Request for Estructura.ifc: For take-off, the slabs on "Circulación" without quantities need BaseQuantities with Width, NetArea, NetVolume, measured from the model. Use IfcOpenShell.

First a look at what the model holds.

```python
import ifcopenshell
import ifcopenshell.util.element
import ifcopenshell.util.unit

model = ifcopenshell.open("Estructura.ifc")
print(model.schema)
for unit_type in ("LENGTHUNIT", "AREAUNIT", "VOLUMEUNIT"):
    print(unit_type, ifcopenshell.util.unit.calculate_unit_scale(model, unit_type))
storey = next(s for s in model.by_type("IfcBuildingStorey") if s.Name == "Circulación")
slabs = [e for e in ifcopenshell.util.element.get_decomposition(storey) if e.is_a("IfcSlab")]
for e in sorted(slabs, key=lambda e: e.id()):
    print(e.id(), e.is_a(), e.Name, list(ifcopenshell.util.element.get_psets(e, qtos_only=True)), sep=" | ")
```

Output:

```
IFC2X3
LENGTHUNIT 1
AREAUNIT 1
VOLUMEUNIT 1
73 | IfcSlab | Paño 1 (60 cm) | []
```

```python
import ifcopenshell
import ifcopenshell.api.pset
import ifcopenshell.geom
import ifcopenshell.util.element
import ifcopenshell.util.shape
import ifcopenshell.util.unit

model = ifcopenshell.open("Estructura.ifc")
unit_scale = ifcopenshell.util.unit.calculate_unit_scale(model)
area_scale = ifcopenshell.util.unit.calculate_unit_scale(model, "AREAUNIT")
volume_scale = ifcopenshell.util.unit.calculate_unit_scale(model, "VOLUMEUNIT")
settings = ifcopenshell.geom.settings()

storey = next(s for s in model.by_type("IfcBuildingStorey") if s.Name == "Circulación")
slabs = [e for e in ifcopenshell.util.element.get_decomposition(storey) if e.is_a("IfcSlab")]

for e in sorted(slabs, key=lambda e: e.id()):
    if ifcopenshell.util.element.get_psets(e, qtos_only=True, should_inherit=False):
        continue
    # Geometry comes back in metres, in the element's own axes.
    shape = ifcopenshell.geom.create_shape(settings, e)
    values = {
        "Width": ifcopenshell.util.shape.get_z(shape.geometry) / unit_scale,
        "NetArea": ifcopenshell.util.shape.get_footprint_area(shape.geometry) / area_scale,
        "NetVolume": ifcopenshell.util.shape.get_volume(shape.geometry) / volume_scale,
    }
    qto = ifcopenshell.api.pset.add_qto(model, product=e, name="BaseQuantities")
    ifcopenshell.api.pset.edit_qto(model, qto=qto, properties=values)
    print(e.id(), {k: round(v, 3) for k, v in values.items()})

model.write("Estructura_rev.ifc")
```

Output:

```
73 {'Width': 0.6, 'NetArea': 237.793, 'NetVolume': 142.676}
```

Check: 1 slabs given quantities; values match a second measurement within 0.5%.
